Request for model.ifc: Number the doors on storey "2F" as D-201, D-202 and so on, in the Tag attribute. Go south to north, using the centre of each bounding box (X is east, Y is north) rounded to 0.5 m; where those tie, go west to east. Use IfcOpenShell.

First a look at what the model holds.

```python
import ifcopenshell
import ifcopenshell.util.element
import ifcopenshell.util.placement

model = ifcopenshell.open("model.ifc")
print(model.schema)
storey = next(s for s in model.by_type("IfcBuildingStorey") if s.Name == "2F")
doors = [e for e in ifcopenshell.util.element.get_decomposition(storey) if e.is_a("IfcDoor")]
for e in sorted(doors, key=lambda e: e.id()):
    origin = ifcopenshell.util.placement.get_local_placement(e.ObjectPlacement)[:3, 3]
    print(e.id(), e.Tag, e.Name, origin.round(2) + 0.0, sep=" | ")
```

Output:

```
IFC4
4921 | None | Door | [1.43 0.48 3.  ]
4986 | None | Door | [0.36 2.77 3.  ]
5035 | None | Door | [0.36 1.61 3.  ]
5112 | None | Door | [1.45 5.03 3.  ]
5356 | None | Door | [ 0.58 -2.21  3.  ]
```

```python
import ifcopenshell
import ifcopenshell.geom
import ifcopenshell.util.element
import ifcopenshell.util.shape

model = ifcopenshell.open("model.ifc")
settings = ifcopenshell.geom.settings()
settings.set("use-world-coords", True)


def centre(element):
    shape = ifcopenshell.geom.create_shape(settings, element)
    return ifcopenshell.util.shape.get_bbox_centroid(shape.geometry)


storey = next(s for s in model.by_type("IfcBuildingStorey") if s.Name == "2F")
doors = [e for e in ifcopenshell.util.element.get_decomposition(storey) if e.is_a("IfcDoor")]

# Insertion points can sit at a corner or the storey origin, so sort by the geometry (in metres).
centres = {e: centre(e) for e in doors}
doors.sort(key=lambda e: (round(centres[e][1] / 0.5), centres[e][0]))

for i, e in enumerate(doors, start=1):
    number = f"D-2{i:02d}"
    e.Tag = number
    print(e.id(), number)

model.write("model_updated.ifc")
```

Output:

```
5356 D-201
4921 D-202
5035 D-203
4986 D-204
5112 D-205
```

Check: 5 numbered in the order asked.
